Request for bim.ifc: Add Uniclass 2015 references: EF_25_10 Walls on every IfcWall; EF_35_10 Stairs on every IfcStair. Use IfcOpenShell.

First a look at what the model holds.

```python
import ifcopenshell

model = ifcopenshell.open("bim.ifc")
print(model.schema)
print("classifications:", [c.Name for c in model.by_type("IfcClassification")])
for ifc_class in ("IfcDoor", "IfcRoof", "IfcStair", "IfcWall", "IfcWindow"):
    print(ifc_class, len(model.by_type(ifc_class)))
```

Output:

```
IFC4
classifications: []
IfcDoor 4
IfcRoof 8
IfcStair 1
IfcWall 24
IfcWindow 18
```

```python
import ifcopenshell
import ifcopenshell.api.classification

model = ifcopenshell.open("bim.ifc")

system = ifcopenshell.api.classification.add_classification(model, classification="Uniclass 2015")

codes = {
    "IfcWall": ("EF_25_10", "Walls"),
    "IfcStair": ("EF_35_10", "Stairs"),
}
for ifc_class, (code, name) in codes.items():
    products = model.by_type(ifc_class)
    ifcopenshell.api.classification.add_reference(
        model, products=products, classification=system, identification=code, name=name
    )
    print(code, len(products))

model.write("bim_updated.ifc")
```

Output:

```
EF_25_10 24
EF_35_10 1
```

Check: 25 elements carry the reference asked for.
